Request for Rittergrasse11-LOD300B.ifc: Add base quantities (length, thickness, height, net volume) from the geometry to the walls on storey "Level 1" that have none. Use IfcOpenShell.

First a look at what the model holds.

```python
import ifcopenshell
import ifcopenshell.util.element
import ifcopenshell.util.unit

model = ifcopenshell.open("Rittergrasse11-LOD300B.ifc")
print(model.schema)
for unit_type in ("LENGTHUNIT", "AREAUNIT", "VOLUMEUNIT"):
    print(unit_type, ifcopenshell.util.unit.calculate_unit_scale(model, unit_type))
storey = next(s for s in model.by_type("IfcBuildingStorey") if s.Name == "Level 1")
walls = [e for e in ifcopenshell.util.element.get_decomposition(storey) if e.is_a("IfcWall")]
for e in sorted(walls, key=lambda e: e.id()):
    print(e.id(), e.is_a(), e.Name, list(ifcopenshell.util.element.get_psets(e, qtos_only=True)), sep=" | ")
```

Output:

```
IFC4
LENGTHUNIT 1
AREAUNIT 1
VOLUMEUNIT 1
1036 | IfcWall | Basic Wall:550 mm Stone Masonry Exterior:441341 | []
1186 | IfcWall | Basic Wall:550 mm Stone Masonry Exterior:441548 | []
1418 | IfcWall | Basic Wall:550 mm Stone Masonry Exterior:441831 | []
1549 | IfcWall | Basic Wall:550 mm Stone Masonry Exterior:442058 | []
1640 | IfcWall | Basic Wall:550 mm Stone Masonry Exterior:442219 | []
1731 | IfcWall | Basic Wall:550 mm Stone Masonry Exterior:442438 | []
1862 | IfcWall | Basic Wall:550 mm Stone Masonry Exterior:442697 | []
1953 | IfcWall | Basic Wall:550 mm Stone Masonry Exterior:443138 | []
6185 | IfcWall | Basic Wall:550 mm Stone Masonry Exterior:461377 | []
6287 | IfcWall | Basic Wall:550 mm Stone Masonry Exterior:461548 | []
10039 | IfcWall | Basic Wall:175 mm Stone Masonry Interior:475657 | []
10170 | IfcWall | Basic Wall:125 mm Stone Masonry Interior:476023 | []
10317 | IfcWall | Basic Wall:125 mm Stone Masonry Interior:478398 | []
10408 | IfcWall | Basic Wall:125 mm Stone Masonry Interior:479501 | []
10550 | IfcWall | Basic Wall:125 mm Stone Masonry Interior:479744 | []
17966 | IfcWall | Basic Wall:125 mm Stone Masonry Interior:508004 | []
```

```python
import ifcopenshell
import ifcopenshell.api.pset
import ifcopenshell.geom
import ifcopenshell.util.element
import ifcopenshell.util.shape
import ifcopenshell.util.unit

model = ifcopenshell.open("Rittergrasse11-LOD300B.ifc")
unit_scale = ifcopenshell.util.unit.calculate_unit_scale(model)
volume_scale = ifcopenshell.util.unit.calculate_unit_scale(model, "VOLUMEUNIT")
settings = ifcopenshell.geom.settings()

storey = next(s for s in model.by_type("IfcBuildingStorey") if s.Name == "Level 1")
walls = [e for e in ifcopenshell.util.element.get_decomposition(storey) if e.is_a("IfcWall")]

for e in sorted(walls, key=lambda e: e.id()):
    if ifcopenshell.util.element.get_psets(e, qtos_only=True, should_inherit=False):
        continue
    # Geometry comes back in metres, in the element's own axes.
    shape = ifcopenshell.geom.create_shape(settings, e)
    values = {
        "Length": ifcopenshell.util.shape.get_x(shape.geometry) / unit_scale,
        "Width": ifcopenshell.util.shape.get_y(shape.geometry) / unit_scale,
        "Height": ifcopenshell.util.shape.get_z(shape.geometry) / unit_scale,
        "NetVolume": ifcopenshell.util.shape.get_volume(shape.geometry) / volume_scale,
    }
    qto = ifcopenshell.api.pset.add_qto(model, product=e, name="Qto_WallBaseQuantities")
    ifcopenshell.api.pset.edit_qto(model, qto=qto, properties=values)
    print(e.id(), {k: round(v, 3) for k, v in values.items()})

model.write("Rittergrasse11-LOD300B_rev.ifc")
```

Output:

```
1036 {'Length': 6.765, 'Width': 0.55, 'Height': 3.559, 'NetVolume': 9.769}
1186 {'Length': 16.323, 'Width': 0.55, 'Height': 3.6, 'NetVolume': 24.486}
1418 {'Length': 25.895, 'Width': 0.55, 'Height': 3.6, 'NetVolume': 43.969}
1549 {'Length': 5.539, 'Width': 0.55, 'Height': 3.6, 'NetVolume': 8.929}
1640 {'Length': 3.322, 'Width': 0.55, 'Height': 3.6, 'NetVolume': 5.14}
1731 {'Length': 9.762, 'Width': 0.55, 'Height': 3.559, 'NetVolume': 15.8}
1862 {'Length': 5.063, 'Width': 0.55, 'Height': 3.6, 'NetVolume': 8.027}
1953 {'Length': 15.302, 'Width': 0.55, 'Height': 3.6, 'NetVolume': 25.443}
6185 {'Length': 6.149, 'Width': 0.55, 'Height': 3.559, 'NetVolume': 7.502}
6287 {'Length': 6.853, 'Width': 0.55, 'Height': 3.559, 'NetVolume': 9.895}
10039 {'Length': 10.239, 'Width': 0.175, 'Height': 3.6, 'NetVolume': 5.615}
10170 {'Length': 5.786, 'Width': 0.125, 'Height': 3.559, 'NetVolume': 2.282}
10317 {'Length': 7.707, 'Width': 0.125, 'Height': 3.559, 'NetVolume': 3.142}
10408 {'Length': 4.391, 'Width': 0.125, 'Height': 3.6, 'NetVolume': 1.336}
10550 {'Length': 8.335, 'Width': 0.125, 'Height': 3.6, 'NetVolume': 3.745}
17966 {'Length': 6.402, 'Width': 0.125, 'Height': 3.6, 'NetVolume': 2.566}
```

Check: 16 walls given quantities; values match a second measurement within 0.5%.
